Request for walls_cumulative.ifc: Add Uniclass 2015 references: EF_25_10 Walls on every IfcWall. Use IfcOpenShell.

First a look at what the model holds.

```python
import ifcopenshell

model = ifcopenshell.open("walls_cumulative.ifc")
print(model.schema)
print("classifications:", [c.Name for c in model.by_type("IfcClassification")])
for ifc_class in ("IfcDoor", "IfcRoof", "IfcStair", "IfcWall", "IfcWindow"):
    print(ifc_class, len(model.by_type(ifc_class)))
```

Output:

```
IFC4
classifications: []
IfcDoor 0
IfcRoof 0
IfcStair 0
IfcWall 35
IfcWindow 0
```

```python
import ifcopenshell
import ifcopenshell.api.classification

model = ifcopenshell.open("walls_cumulative.ifc")

system = ifcopenshell.api.classification.add_classification(model, classification="Uniclass 2015")

codes = {
    "IfcWall": ("EF_25_10", "Walls"),
}
for ifc_class, (code, name) in codes.items():
    products = model.by_type(ifc_class)
    ifcopenshell.api.classification.add_reference(
        model, products=products, classification=system, identification=code, name=name
    )
    print(code, len(products))

model.write("walls_cumulative_updated.ifc")
```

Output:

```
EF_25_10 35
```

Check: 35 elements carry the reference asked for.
